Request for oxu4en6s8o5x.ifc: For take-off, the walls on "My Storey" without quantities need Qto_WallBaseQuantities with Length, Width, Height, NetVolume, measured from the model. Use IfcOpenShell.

First a look at what the model holds.

```python
import ifcopenshell
import ifcopenshell.util.element
import ifcopenshell.util.unit

model = ifcopenshell.open("oxu4en6s8o5x.ifc")
print(model.schema)
for unit_type in ("LENGTHUNIT", "AREAUNIT", "VOLUMEUNIT"):
    print(unit_type, ifcopenshell.util.unit.calculate_unit_scale(model, unit_type))
storey = next(s for s in model.by_type("IfcBuildingStorey") if s.Name == "My Storey")
walls = [e for e in ifcopenshell.util.element.get_decomposition(storey) if e.is_a("IfcWall")]
for e in sorted(walls, key=lambda e: e.id()):
    print(e.id(), e.is_a(), e.Name, list(ifcopenshell.util.element.get_psets(e, qtos_only=True)), sep=" | ")
```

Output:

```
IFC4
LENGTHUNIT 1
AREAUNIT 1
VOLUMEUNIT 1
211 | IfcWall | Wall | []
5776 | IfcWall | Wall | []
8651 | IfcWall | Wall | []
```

```python
import ifcopenshell
import ifcopenshell.api.pset
import ifcopenshell.geom
import ifcopenshell.util.element
import ifcopenshell.util.shape
import ifcopenshell.util.unit

model = ifcopenshell.open("oxu4en6s8o5x.ifc")
unit_scale = ifcopenshell.util.unit.calculate_unit_scale(model)
volume_scale = ifcopenshell.util.unit.calculate_unit_scale(model, "VOLUMEUNIT")
settings = ifcopenshell.geom.settings()

storey = next(s for s in model.by_type("IfcBuildingStorey") if s.Name == "My Storey")
walls = [e for e in ifcopenshell.util.element.get_decomposition(storey) if e.is_a("IfcWall")]

for e in sorted(walls, key=lambda e: e.id()):
    if ifcopenshell.util.element.get_psets(e, qtos_only=True, should_inherit=False):
        continue
    # Geometry comes back in metres, in the element's own axes.
    shape = ifcopenshell.geom.create_shape(settings, e)
    values = {
        "Length": ifcopenshell.util.shape.get_x(shape.geometry) / unit_scale,
        "Width": ifcopenshell.util.shape.get_y(shape.geometry) / unit_scale,
        "Height": ifcopenshell.util.shape.get_z(shape.geometry) / unit_scale,
        "NetVolume": ifcopenshell.util.shape.get_volume(shape.geometry) / volume_scale,
    }
    qto = ifcopenshell.api.pset.add_qto(model, product=e, name="Qto_WallBaseQuantities")
    ifcopenshell.api.pset.edit_qto(model, qto=qto, properties=values)
    print(e.id(), {k: round(v, 3) for k, v in values.items()})

model.write("oxu4en6s8o5x_updated.ifc")
```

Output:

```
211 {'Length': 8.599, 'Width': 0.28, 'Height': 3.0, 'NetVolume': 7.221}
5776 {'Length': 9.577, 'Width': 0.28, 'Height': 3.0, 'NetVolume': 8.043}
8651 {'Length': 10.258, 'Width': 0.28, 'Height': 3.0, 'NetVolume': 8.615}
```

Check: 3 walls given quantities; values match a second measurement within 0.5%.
